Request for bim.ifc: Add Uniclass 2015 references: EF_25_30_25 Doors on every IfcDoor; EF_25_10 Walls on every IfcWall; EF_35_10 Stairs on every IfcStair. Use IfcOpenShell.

First a look at what the model holds.

```python
import ifcopenshell

model = ifcopenshell.open("bim.ifc")
print(model.schema)
print("classifications:", [c.Name for c in model.by_type("IfcClassification")])
for ifc_class in ("IfcDoor", "IfcRoof", "IfcStair", "IfcWall", "IfcWindow"):
    print(ifc_class, len(model.by_type(ifc_class)))
```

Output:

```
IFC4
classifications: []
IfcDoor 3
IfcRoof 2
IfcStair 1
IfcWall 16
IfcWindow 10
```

```python
import ifcopenshell
import ifcopenshell.api.classification

model = ifcopenshell.open("bim.ifc")

system = ifcopenshell.api.classification.add_classification(model, classification="Uniclass 2015")

codes = {
    "IfcDoor": ("EF_25_30_25", "Doors"),
    "IfcWall": ("EF_25_10", "Walls"),
    "IfcStair": ("EF_35_10", "Stairs"),
}
for ifc_class, (code, name) in codes.items():
    products = model.by_type(ifc_class)
    ifcopenshell.api.classification.add_reference(
        model, products=products, classification=system, identification=code, name=name
    )
    print(code, len(products))

model.write("bim_v2.ifc")
```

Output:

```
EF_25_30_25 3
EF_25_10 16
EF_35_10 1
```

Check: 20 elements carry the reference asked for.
